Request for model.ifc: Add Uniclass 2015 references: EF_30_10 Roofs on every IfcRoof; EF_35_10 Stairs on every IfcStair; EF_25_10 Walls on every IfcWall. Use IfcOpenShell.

First a look at what the model holds.

```python
import ifcopenshell

model = ifcopenshell.open("model.ifc")
print(model.schema)
print("classifications:", [c.Name for c in model.by_type("IfcClassification")])
for ifc_class in ("IfcDoor", "IfcRoof", "IfcStair", "IfcWall", "IfcWindow"):
    print(ifc_class, len(model.by_type(ifc_class)))
```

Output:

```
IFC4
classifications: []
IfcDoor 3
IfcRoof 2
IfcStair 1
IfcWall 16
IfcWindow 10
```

```python
import ifcopenshell
import ifcopenshell.api.classification

model = ifcopenshell.open("model.ifc")

system = ifcopenshell.api.classification.add_classification(model, classification="Uniclass 2015")

codes = {
    "IfcRoof": ("EF_30_10", "Roofs"),
    "IfcStair": ("EF_35_10", "Stairs"),
    "IfcWall": ("EF_25_10", "Walls"),
}
for ifc_class, (code, name) in codes.items():
    products = model.by_type(ifc_class)
    ifcopenshell.api.classification.add_reference(
        model, products=products, classification=system, identification=code, name=name
    )
    print(code, len(products))

model.write("model_edited.ifc")
```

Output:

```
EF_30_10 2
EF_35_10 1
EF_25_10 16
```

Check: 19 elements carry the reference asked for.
